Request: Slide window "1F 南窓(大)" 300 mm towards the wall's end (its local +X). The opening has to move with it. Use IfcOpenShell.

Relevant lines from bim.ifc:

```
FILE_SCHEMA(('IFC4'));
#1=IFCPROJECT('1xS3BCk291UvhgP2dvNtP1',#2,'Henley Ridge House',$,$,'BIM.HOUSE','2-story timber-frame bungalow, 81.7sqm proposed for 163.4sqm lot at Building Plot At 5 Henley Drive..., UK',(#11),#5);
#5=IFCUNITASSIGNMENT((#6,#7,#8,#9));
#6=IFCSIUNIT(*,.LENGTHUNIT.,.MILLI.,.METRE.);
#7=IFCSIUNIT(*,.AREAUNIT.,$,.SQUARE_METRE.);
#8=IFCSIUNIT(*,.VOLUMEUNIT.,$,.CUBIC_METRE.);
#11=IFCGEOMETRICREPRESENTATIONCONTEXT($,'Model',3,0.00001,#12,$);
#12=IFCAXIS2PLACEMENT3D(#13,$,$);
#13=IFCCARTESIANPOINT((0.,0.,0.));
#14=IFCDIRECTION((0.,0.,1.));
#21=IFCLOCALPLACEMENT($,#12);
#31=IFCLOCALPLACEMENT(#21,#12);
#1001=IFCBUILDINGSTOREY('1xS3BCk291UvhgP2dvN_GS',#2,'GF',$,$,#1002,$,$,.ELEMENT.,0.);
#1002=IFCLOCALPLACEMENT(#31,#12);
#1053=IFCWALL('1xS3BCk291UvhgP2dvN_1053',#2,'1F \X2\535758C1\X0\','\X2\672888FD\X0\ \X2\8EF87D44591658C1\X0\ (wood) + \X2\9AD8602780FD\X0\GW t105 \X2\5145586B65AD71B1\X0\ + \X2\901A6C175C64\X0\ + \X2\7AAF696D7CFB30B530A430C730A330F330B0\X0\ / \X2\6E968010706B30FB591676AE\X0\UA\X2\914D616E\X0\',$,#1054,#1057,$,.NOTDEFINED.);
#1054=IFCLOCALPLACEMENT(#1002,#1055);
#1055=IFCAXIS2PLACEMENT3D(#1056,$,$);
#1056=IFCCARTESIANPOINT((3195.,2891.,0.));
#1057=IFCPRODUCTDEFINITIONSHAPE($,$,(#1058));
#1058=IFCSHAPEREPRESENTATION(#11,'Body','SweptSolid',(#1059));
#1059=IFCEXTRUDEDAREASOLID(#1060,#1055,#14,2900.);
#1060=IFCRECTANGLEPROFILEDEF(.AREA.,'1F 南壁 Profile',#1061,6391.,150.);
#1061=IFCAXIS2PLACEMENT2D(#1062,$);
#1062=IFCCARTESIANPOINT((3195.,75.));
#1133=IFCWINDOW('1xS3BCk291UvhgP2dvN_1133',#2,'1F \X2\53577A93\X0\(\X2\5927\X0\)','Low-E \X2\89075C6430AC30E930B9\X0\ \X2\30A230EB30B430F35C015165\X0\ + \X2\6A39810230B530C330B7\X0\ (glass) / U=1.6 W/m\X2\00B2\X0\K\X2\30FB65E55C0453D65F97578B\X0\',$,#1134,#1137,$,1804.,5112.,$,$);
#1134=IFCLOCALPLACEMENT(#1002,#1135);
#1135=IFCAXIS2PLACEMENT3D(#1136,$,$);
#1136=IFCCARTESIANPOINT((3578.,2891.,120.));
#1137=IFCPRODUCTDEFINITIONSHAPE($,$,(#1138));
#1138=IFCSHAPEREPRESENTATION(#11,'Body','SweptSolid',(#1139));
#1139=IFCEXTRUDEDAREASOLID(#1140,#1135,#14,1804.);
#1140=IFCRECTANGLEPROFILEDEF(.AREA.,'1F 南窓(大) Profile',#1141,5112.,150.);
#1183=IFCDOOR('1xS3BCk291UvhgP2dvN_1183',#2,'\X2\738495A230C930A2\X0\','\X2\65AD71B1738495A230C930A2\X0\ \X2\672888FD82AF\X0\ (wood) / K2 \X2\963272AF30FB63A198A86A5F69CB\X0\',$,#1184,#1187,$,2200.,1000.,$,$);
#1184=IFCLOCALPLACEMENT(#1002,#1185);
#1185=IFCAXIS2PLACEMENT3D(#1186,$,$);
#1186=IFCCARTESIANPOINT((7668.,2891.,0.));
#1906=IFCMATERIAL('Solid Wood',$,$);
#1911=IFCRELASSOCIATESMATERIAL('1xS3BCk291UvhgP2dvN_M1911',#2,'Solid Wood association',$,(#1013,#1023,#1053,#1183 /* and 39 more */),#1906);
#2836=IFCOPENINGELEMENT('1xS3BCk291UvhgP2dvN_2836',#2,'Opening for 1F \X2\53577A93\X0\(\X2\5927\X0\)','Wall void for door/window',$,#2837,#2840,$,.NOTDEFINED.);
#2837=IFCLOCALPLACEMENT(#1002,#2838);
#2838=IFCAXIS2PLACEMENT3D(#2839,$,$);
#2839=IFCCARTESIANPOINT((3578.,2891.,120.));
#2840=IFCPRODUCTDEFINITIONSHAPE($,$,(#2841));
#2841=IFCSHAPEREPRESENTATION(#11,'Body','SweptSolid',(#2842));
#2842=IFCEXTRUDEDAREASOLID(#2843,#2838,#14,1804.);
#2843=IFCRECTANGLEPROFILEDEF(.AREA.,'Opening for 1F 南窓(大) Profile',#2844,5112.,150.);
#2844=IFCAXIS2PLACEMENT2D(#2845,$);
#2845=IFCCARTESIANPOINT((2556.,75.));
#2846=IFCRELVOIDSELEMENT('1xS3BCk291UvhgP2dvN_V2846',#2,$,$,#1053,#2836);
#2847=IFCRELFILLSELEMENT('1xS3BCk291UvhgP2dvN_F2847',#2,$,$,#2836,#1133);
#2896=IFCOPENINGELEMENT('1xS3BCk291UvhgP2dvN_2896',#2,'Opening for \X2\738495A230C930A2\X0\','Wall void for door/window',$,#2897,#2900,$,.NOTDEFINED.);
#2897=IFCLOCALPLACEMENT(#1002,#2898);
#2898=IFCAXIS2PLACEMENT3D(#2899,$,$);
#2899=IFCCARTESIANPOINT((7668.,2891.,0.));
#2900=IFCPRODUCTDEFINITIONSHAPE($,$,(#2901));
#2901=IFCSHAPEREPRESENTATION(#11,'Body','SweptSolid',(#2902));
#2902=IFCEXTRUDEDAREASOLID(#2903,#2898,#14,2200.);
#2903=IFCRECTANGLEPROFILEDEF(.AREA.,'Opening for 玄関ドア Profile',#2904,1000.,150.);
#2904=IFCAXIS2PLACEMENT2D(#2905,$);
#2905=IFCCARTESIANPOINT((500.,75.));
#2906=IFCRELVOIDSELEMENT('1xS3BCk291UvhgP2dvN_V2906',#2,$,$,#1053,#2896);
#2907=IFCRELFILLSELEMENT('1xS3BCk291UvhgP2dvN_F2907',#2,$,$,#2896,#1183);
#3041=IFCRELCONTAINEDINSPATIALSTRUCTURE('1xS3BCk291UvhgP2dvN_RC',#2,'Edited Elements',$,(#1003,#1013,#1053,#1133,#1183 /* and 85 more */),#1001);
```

```python
import ifcopenshell
import ifcopenshell.api.geometry
import ifcopenshell.util.placement

model = ifcopenshell.open("bim.ifc")

window = model.by_guid("1xS3BCk291UvhgP2dvN_1133")
opening = window.FillsVoids[0].RelatingOpeningElement
wall = opening.VoidsElements[0].RelatingBuildingElement

wall_matrix = ifcopenshell.util.placement.get_local_placement(wall.ObjectPlacement)
shift = wall_matrix[:3, 0] * 300.0
before = ifcopenshell.util.placement.get_local_placement(window.ObjectPlacement)[:3, 3].copy()

# The window is not placed relative to its opening, so move both.
for product in (opening, window):
    matrix = ifcopenshell.util.placement.get_local_placement(product.ObjectPlacement)
    matrix[:3, 3] += shift
    ifcopenshell.api.geometry.edit_object_placement(model, product=product, matrix=matrix, is_si=False)

after = ifcopenshell.util.placement.get_local_placement(window.ObjectPlacement)[:3, 3]
print("window moved by", (after - before).round(3) + 0.0)

model.write("bim_updated.ifc")
```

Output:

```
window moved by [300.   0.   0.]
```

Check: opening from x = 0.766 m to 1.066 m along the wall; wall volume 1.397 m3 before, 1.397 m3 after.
